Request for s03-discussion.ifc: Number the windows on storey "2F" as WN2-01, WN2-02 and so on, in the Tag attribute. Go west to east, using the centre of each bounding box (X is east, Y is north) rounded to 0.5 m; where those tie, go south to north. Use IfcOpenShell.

First a look at what the model holds.

```python
import ifcopenshell
import ifcopenshell.util.element
import ifcopenshell.util.placement

model = ifcopenshell.open("s03-discussion.ifc")
print(model.schema)
storey = next(s for s in model.by_type("IfcBuildingStorey") if s.Name == "2F")
windows = [e for e in ifcopenshell.util.element.get_decomposition(storey) if e.is_a("IfcWindow")]
for e in sorted(windows, key=lambda e: e.id()):
    origin = ifcopenshell.util.placement.get_local_placement(e.ObjectPlacement)[:3, 3]
    print(e.id(), e.Tag, e.Name, origin.round(2) + 0.0, sep=" | ")
```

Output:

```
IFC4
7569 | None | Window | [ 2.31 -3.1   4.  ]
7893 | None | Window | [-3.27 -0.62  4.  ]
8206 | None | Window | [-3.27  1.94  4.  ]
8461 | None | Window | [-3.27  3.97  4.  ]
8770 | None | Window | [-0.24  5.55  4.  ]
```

```python
import ifcopenshell
import ifcopenshell.geom
import ifcopenshell.util.element
import ifcopenshell.util.shape

model = ifcopenshell.open("s03-discussion.ifc")
settings = ifcopenshell.geom.settings()
settings.set("use-world-coords", True)


def centre(element):
    shape = ifcopenshell.geom.create_shape(settings, element)
    return ifcopenshell.util.shape.get_bbox_centroid(shape.geometry)


storey = next(s for s in model.by_type("IfcBuildingStorey") if s.Name == "2F")
windows = [e for e in ifcopenshell.util.element.get_decomposition(storey) if e.is_a("IfcWindow")]

# Insertion points can sit at a corner or the storey origin, so sort by the geometry (in metres).
centres = {e: centre(e) for e in windows}
windows.sort(key=lambda e: (round(centres[e][0] / 0.5), centres[e][1]))

for i, e in enumerate(windows, start=1):
    number = f"WN2-{i:02d}"
    e.Tag = number
    print(e.id(), number)

model.write("s03-discussion_v2.ifc")
```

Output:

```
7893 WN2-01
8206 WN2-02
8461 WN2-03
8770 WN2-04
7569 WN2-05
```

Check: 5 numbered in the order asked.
